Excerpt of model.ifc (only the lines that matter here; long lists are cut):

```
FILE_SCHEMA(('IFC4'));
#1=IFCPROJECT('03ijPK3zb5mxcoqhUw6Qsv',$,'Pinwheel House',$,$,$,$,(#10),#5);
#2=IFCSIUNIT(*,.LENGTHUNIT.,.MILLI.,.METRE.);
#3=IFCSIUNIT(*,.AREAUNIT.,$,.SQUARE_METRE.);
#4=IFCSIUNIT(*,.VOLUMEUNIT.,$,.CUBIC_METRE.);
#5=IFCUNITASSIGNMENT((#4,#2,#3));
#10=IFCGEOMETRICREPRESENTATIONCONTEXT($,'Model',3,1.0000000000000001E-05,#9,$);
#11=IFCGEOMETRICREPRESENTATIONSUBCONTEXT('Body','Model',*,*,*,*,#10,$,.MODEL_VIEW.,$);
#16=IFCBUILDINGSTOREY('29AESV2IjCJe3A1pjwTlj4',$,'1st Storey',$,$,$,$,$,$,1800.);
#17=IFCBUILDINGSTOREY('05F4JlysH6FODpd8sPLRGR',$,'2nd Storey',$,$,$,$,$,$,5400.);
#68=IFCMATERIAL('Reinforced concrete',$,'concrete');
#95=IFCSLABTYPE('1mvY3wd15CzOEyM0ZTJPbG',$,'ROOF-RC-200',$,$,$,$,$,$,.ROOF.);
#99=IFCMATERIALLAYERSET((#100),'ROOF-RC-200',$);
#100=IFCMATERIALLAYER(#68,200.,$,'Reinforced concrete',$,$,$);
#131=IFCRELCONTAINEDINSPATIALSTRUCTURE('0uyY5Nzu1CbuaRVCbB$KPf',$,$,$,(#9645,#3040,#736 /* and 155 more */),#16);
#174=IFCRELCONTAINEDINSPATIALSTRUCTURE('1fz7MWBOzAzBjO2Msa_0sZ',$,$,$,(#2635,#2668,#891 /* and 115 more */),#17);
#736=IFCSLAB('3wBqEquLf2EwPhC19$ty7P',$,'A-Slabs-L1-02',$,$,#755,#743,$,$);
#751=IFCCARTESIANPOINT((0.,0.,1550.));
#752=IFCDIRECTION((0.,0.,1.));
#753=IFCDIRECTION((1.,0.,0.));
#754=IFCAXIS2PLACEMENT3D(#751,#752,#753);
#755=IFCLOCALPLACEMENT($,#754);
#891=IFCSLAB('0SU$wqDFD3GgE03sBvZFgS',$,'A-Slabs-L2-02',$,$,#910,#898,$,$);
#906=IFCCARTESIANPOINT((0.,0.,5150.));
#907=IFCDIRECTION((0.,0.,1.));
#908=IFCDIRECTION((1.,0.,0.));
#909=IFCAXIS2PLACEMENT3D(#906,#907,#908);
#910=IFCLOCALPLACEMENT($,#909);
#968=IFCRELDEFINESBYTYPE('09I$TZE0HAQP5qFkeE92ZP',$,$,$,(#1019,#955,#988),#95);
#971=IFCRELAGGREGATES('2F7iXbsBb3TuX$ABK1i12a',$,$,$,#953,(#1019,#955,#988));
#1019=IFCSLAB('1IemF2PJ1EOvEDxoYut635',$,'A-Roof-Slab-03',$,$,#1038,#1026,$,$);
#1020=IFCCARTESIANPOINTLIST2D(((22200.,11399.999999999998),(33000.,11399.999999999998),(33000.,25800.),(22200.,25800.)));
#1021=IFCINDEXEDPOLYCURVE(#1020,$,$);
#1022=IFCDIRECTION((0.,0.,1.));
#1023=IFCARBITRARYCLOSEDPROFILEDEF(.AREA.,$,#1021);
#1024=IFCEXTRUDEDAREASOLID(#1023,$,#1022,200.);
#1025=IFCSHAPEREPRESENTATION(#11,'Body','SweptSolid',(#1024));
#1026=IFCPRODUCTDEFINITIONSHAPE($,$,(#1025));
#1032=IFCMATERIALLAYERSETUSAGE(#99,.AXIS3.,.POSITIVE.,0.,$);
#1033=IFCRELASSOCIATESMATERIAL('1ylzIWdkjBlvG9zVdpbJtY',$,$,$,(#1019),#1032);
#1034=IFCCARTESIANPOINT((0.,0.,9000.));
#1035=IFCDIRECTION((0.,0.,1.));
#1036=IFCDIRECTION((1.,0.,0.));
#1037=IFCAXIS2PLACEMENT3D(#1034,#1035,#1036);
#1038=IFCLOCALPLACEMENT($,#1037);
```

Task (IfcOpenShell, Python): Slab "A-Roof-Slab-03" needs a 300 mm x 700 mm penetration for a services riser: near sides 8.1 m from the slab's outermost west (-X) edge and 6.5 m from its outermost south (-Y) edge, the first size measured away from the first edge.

```python
import numpy as np
import ifcopenshell
import ifcopenshell.api.feature
import ifcopenshell.api.geometry
import ifcopenshell.api.root
import ifcopenshell.geom
import ifcopenshell.util.placement
import ifcopenshell.util.representation
import ifcopenshell.util.shape
import ifcopenshell.util.unit

model = ifcopenshell.open("model.ifc")
unit_scale = ifcopenshell.util.unit.calculate_unit_scale(model)
settings = ifcopenshell.geom.settings()


def volume(element):
    """Net volume in cubic metres, openings subtracted."""
    shape = ifcopenshell.geom.create_shape(settings, element)
    return ifcopenshell.util.shape.get_volume(shape.geometry)


slab = model.by_id(1019)
before = volume(slab)

# Extent in the slab's own axes, in metres. The edges named are its -X and -Y sides.
slab_shape = ifcopenshell.geom.create_shape(settings, slab)
vertices = ifcopenshell.util.shape.get_vertices(slab_shape.geometry)
x_min, y_min, bottom = vertices.min(axis=0)
top = vertices[:, 2].max()

opening = ifcopenshell.api.root.create_entity(model, ifc_class="IfcOpeningElement", name="Services riser opening", predefined_type="OPENING")
context = ifcopenshell.util.representation.get_context(model, "Model", "Body", "MODEL_VIEW")
width, depth = 0.3, 0.7
outline = [(0.0, 0.0), (width, 0.0), (width, depth), (0.0, depth), (0.0, 0.0)]
# Overshoot both faces by 50 mm so the cut is clean.
shape = ifcopenshell.api.geometry.add_slab_representation(
    model, context=context, depth=top - bottom + 0.1, polyline=outline
)
ifcopenshell.api.geometry.assign_representation(model, product=opening, representation=shape)

matrix = ifcopenshell.util.placement.get_local_placement(slab.ObjectPlacement)
matrix[:, 3] = matrix @ np.append(np.array([x_min + 8.1, y_min + 6.5, bottom - 0.05]) / unit_scale, 1.0)
ifcopenshell.api.geometry.edit_object_placement(model, product=opening, matrix=matrix, is_si=False)
ifcopenshell.api.feature.add_feature(model, feature=opening, element=slab)

after = volume(slab)

print(f"slab volume {before:.3f} -> {after:.3f} m3")

model.write("model-out.ifc")
```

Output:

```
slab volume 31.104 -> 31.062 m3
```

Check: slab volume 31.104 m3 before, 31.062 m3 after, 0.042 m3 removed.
